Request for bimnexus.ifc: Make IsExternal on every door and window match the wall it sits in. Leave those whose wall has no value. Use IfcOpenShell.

First a look at what the model holds.

```python
import ifcopenshell
import ifcopenshell.util.element

model = ifcopenshell.open("bimnexus.ifc")
print(model.schema)
seen = {}
for e in model.by_type("IfcDoor") + model.by_type("IfcWindow"):
    if not e.FillsVoids:
        continue
    host = e.FillsVoids[0].RelatingOpeningElement.VoidsElements[0].RelatingBuildingElement
    own = ifcopenshell.util.element.get_pset(e, f"Pset_{e.is_a()[3:].removesuffix('StandardCase')}Common", "IsExternal")
    wall = ifcopenshell.util.element.get_pset(host, "Pset_WallCommon", "IsExternal")
    seen[e.is_a(), own, wall] = seen.get((e.is_a(), own, wall), 0) + 1
for (cls, own, wall), count in sorted(seen.items(), key=str):
    print(count, cls, "IsExternal:", own, "| host wall:", wall)
```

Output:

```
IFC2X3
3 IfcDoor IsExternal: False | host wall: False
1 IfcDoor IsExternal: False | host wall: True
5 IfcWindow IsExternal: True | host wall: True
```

```python
import ifcopenshell
import ifcopenshell.api.pset
import ifcopenshell.util.element

model = ifcopenshell.open("bimnexus.ifc")

count = 0
for ifc_class, pset_name in (("IfcDoor", "Pset_DoorCommon"), ("IfcWindow", "Pset_WindowCommon")):
    for e in model.by_type(ifc_class):
        if not e.FillsVoids:
            continue
        host = e.FillsVoids[0].RelatingOpeningElement.VoidsElements[0].RelatingBuildingElement
        external = ifcopenshell.util.element.get_pset(host, "Pset_WallCommon", "IsExternal")
        if external is None or ifcopenshell.util.element.get_pset(e, pset_name, "IsExternal") == external:
            continue
        pset = ifcopenshell.api.pset.add_pset(model, product=e, name=pset_name)
        ifcopenshell.api.pset.edit_pset(model, pset=pset, properties={"IsExternal": external})
        count += 1

print(count, "updated")

model.write("bimnexus_v2.ifc")
```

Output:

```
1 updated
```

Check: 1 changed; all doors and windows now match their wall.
